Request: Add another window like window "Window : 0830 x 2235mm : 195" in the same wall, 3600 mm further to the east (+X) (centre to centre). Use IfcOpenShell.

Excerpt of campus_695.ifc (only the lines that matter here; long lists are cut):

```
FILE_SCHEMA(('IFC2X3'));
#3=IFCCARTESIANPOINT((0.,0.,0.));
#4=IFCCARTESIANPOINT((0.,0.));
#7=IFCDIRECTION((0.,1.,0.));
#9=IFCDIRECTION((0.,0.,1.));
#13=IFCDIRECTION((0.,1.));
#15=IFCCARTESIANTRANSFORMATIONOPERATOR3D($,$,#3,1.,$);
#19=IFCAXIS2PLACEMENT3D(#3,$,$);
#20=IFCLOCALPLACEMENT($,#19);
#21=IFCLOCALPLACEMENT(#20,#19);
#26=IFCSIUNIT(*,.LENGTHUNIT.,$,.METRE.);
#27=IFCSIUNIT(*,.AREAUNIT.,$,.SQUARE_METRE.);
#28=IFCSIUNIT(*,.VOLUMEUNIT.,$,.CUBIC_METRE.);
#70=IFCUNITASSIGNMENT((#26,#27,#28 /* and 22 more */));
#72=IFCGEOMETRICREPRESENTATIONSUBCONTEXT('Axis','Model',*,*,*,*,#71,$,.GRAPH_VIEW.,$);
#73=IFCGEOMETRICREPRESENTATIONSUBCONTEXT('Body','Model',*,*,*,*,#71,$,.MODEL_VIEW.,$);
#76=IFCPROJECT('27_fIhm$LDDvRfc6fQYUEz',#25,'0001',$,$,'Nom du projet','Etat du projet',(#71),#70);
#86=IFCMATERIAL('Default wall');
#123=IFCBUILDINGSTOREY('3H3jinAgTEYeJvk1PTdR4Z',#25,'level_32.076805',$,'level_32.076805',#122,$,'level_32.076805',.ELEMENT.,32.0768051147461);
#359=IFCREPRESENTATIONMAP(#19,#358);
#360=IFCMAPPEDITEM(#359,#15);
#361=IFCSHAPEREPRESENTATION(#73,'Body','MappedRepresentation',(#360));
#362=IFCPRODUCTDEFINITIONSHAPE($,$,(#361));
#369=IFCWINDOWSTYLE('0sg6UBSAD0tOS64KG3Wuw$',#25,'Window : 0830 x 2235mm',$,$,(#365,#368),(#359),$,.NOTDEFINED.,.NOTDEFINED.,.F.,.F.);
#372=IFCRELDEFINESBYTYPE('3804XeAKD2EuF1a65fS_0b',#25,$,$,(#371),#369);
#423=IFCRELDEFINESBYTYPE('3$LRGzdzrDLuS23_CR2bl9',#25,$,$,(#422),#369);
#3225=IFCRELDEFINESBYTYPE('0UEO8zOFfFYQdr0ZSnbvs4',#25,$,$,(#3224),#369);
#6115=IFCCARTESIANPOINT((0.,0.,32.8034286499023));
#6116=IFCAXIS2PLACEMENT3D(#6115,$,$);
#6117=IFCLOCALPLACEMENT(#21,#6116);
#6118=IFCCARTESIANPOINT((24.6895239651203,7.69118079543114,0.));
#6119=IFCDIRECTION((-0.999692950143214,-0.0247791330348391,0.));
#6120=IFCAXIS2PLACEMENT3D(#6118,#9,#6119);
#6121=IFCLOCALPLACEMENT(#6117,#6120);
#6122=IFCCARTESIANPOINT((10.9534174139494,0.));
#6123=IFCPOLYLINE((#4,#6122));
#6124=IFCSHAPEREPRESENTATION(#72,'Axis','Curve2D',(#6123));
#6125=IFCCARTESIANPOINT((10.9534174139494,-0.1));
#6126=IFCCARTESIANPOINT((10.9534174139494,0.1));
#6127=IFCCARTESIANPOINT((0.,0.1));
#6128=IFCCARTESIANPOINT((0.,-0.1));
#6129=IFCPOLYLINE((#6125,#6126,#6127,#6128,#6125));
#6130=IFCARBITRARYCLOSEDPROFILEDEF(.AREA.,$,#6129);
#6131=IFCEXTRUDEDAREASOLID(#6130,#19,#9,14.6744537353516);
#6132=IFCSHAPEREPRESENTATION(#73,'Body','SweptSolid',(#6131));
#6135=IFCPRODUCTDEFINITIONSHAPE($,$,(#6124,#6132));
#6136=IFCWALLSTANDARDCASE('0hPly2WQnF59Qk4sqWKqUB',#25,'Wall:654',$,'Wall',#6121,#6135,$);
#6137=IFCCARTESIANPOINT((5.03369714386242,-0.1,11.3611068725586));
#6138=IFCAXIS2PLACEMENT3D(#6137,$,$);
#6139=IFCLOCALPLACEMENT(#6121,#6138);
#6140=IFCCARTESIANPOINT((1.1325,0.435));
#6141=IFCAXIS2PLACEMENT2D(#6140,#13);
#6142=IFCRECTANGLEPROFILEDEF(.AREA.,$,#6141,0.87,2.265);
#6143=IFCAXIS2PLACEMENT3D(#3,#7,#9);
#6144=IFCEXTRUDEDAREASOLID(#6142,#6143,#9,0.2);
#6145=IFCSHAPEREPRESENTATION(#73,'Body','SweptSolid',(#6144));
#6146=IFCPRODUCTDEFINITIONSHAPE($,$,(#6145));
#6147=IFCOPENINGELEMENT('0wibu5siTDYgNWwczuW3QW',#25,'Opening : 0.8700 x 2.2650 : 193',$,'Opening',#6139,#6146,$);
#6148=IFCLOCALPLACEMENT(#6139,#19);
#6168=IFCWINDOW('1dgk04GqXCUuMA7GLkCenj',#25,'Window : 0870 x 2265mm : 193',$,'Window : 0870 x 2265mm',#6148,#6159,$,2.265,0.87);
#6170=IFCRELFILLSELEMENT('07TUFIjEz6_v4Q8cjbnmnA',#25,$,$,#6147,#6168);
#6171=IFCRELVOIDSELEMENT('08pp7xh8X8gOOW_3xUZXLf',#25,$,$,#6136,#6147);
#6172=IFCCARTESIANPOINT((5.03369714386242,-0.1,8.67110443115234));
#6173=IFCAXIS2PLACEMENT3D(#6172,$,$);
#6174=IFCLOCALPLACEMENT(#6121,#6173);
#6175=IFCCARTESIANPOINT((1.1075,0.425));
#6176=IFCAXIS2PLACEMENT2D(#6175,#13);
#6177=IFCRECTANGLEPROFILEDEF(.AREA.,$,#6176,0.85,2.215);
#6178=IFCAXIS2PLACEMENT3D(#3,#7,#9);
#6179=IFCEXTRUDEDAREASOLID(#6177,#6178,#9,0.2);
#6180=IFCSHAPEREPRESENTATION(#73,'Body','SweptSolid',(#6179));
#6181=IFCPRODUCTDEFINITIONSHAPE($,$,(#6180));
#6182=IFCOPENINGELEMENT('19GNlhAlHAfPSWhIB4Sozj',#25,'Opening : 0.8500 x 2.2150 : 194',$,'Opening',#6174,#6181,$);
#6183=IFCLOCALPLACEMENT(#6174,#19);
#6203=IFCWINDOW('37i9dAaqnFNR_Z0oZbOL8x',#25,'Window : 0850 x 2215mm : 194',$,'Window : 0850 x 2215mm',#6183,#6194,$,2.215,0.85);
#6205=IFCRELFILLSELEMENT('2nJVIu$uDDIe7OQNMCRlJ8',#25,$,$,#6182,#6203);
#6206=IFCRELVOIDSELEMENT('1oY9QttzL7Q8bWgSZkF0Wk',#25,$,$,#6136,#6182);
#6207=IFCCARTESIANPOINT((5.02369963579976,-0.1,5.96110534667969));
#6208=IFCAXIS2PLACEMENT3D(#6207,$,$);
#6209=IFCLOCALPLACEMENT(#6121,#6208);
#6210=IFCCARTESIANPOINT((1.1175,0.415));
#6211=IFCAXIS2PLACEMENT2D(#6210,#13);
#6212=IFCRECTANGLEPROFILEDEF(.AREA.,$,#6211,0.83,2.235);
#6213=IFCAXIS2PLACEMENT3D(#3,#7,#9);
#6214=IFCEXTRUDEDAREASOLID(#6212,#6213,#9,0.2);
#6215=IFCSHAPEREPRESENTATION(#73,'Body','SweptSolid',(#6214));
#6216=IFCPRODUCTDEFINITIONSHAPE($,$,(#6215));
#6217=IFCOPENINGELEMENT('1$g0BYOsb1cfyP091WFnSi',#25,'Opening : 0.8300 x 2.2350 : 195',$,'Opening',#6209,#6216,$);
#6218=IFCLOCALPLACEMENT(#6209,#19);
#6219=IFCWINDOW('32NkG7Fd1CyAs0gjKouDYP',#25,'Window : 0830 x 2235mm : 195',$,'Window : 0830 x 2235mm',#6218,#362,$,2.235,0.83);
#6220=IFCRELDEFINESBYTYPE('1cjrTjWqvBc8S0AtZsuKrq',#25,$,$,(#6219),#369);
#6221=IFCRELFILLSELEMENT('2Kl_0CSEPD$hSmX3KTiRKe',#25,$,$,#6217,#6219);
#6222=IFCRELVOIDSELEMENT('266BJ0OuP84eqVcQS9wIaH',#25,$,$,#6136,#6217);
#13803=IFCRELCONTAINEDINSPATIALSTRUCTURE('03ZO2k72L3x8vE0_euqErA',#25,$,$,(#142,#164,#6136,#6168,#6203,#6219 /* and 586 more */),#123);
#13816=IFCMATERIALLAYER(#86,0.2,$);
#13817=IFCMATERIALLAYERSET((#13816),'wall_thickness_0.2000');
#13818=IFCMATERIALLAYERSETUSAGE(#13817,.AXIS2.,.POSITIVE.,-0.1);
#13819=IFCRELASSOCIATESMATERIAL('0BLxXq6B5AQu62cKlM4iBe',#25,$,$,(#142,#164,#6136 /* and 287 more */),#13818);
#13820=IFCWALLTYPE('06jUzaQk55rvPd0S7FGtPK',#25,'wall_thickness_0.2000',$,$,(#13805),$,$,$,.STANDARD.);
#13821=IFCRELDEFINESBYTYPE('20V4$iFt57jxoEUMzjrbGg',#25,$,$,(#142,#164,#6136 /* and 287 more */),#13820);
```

```python
import ifcopenshell
import ifcopenshell.api.feature
import ifcopenshell.api.geometry
import ifcopenshell.api.root
import ifcopenshell.geom
import ifcopenshell.util.element
import ifcopenshell.util.placement
import ifcopenshell.util.shape

model = ifcopenshell.open("campus_695.ifc")
settings = ifcopenshell.geom.settings()


def volume(element):
    """Net volume in cubic metres, openings subtracted."""
    shape = ifcopenshell.geom.create_shape(settings, element)
    return ifcopenshell.util.shape.get_volume(shape.geometry)


window = model.by_guid("32NkG7Fd1CyAs0gjKouDYP")
opening = window.FillsVoids[0].RelatingOpeningElement
wall = opening.VoidsElements[0].RelatingBuildingElement
before = volume(wall)
shift = ifcopenshell.util.placement.get_local_placement(wall.ObjectPlacement)[:3, 0] * -3.6

# copy_class copies the void relationship, type, container and properties, but no geometry.
new_opening = ifcopenshell.api.root.copy_class(model, product=opening)
new_opening.Representation = ifcopenshell.util.element.copy_deep(
    model, opening.Representation, exclude=["IfcGeometricRepresentationContext", "IfcRepresentationMap"]
)
new_opening.Name = "Opening : 0.8300 x 2.2350"
new_window = ifcopenshell.api.root.copy_class(model, product=window)
new_window.Representation = ifcopenshell.util.element.copy_deep(
    model, window.Representation, exclude=["IfcGeometricRepresentationContext", "IfcRepresentationMap"]
)
new_window.Name = "Window : 0830 x 2235mm"
fills = ifcopenshell.api.feature.add_filling(model, opening=new_opening, element=new_window)
fills.OwnerHistory = new_window.OwnerHistory  # required in IFC2X3

for old, new in ((opening, new_opening), (window, new_window)):
    matrix = ifcopenshell.util.placement.get_local_placement(old.ObjectPlacement)
    matrix[:3, 3] += shift
    ifcopenshell.api.geometry.edit_object_placement(model, product=new, matrix=matrix, is_si=False)

after = volume(wall)

print(f"wall volume {before:.3f} -> {after:.3f} m3")

model.write("campus_695_v2.ifc")
```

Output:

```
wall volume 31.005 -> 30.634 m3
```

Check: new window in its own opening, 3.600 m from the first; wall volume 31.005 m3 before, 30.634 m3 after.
